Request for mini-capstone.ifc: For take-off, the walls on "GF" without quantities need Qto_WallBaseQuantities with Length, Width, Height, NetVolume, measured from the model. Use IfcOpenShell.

First a look at what the model holds.

```python
import ifcopenshell
import ifcopenshell.util.element
import ifcopenshell.util.unit

model = ifcopenshell.open("mini-capstone.ifc")
print(model.schema)
for unit_type in ("LENGTHUNIT", "AREAUNIT", "VOLUMEUNIT"):
    print(unit_type, ifcopenshell.util.unit.calculate_unit_scale(model, unit_type))
storey = next(s for s in model.by_type("IfcBuildingStorey") if s.Name == "GF")
walls = [e for e in ifcopenshell.util.element.get_decomposition(storey) if e.is_a("IfcWall")]
for e in sorted(walls, key=lambda e: e.id()):
    print(e.id(), e.is_a(), e.Name, list(ifcopenshell.util.element.get_psets(e, qtos_only=True)), sep=" | ")
```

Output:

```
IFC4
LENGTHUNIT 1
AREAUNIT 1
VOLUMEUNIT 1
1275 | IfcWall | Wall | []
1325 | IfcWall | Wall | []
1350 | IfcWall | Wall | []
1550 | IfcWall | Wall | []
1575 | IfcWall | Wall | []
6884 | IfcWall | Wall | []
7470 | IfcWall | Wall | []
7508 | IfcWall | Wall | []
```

```python
import ifcopenshell
import ifcopenshell.api.pset
import ifcopenshell.geom
import ifcopenshell.util.element
import ifcopenshell.util.shape
import ifcopenshell.util.unit

model = ifcopenshell.open("mini-capstone.ifc")
unit_scale = ifcopenshell.util.unit.calculate_unit_scale(model)
volume_scale = ifcopenshell.util.unit.calculate_unit_scale(model, "VOLUMEUNIT")
settings = ifcopenshell.geom.settings()

storey = next(s for s in model.by_type("IfcBuildingStorey") if s.Name == "GF")
walls = [e for e in ifcopenshell.util.element.get_decomposition(storey) if e.is_a("IfcWall")]

for e in sorted(walls, key=lambda e: e.id()):
    if ifcopenshell.util.element.get_psets(e, qtos_only=True, should_inherit=False):
        continue
    # Geometry comes back in metres, in the element's own axes.
    shape = ifcopenshell.geom.create_shape(settings, e)
    values = {
        "Length": ifcopenshell.util.shape.get_x(shape.geometry) / unit_scale,
        "Width": ifcopenshell.util.shape.get_y(shape.geometry) / unit_scale,
        "Height": ifcopenshell.util.shape.get_z(shape.geometry) / unit_scale,
        "NetVolume": ifcopenshell.util.shape.get_volume(shape.geometry) / volume_scale,
    }
    qto = ifcopenshell.api.pset.add_qto(model, product=e, name="Qto_WallBaseQuantities")
    ifcopenshell.api.pset.edit_qto(model, qto=qto, properties=values)
    print(e.id(), {k: round(v, 3) for k, v in values.items()})

model.write("mini-capstone_rev.ifc")
```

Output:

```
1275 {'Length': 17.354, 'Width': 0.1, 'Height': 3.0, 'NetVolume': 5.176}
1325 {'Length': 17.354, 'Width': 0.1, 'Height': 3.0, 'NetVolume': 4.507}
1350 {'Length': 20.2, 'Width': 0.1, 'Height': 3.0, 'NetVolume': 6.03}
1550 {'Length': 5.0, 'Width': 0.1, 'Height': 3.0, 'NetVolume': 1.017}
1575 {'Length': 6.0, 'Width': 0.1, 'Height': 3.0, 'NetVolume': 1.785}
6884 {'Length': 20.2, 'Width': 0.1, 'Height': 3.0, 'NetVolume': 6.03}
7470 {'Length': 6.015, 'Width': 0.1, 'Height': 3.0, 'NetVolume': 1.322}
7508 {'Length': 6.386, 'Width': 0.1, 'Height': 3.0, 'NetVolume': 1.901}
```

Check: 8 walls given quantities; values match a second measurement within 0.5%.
